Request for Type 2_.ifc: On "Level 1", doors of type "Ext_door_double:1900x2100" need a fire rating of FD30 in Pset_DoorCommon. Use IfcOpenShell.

First a look at what the model holds.

```python
import ifcopenshell
import ifcopenshell.util.element

model = ifcopenshell.open("Type 2_.ifc")
print(model.schema)
storey = next(s for s in model.by_type("IfcBuildingStorey") if s.Name == "Level 1")
doors = [e for e in ifcopenshell.util.element.get_decomposition(storey) if e.is_a("IfcDoor")]
seen = {}
for e in doors:
    element_type = ifcopenshell.util.element.get_type(e)
    key = (element_type.Name if element_type != e and element_type else None, ifcopenshell.util.element.get_pset(e, "Pset_DoorCommon", "FireRating"))
    seen[key] = seen.get(key, 0) + 1
for (name, value), count in sorted(seen.items(), key=str):
    print(count, "x", name, "|", value)
```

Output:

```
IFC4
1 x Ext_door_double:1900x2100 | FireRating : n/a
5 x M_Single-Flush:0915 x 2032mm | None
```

```python
import ifcopenshell
import ifcopenshell.api.pset
import ifcopenshell.util.element

model = ifcopenshell.open("Type 2_.ifc")

storey = next(s for s in model.by_type("IfcBuildingStorey") if s.Name == "Level 1")
doors = [e for e in ifcopenshell.util.element.get_decomposition(storey) if e.is_a("IfcDoor")]

count = 0
for e in doors:
    element_type = ifcopenshell.util.element.get_type(e)
    if element_type in (None, e) or element_type.Name != "Ext_door_double:1900x2100":
        continue
    # add_pset returns the element's existing set when there is one.
    pset = ifcopenshell.api.pset.add_pset(model, product=e, name="Pset_DoorCommon")
    ifcopenshell.api.pset.edit_pset(model, pset=pset, properties={"FireRating": "FD30"})
    count += 1

print(count, "doors updated")

model.write("Type 2__rev.ifc")
```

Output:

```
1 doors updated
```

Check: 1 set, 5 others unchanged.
